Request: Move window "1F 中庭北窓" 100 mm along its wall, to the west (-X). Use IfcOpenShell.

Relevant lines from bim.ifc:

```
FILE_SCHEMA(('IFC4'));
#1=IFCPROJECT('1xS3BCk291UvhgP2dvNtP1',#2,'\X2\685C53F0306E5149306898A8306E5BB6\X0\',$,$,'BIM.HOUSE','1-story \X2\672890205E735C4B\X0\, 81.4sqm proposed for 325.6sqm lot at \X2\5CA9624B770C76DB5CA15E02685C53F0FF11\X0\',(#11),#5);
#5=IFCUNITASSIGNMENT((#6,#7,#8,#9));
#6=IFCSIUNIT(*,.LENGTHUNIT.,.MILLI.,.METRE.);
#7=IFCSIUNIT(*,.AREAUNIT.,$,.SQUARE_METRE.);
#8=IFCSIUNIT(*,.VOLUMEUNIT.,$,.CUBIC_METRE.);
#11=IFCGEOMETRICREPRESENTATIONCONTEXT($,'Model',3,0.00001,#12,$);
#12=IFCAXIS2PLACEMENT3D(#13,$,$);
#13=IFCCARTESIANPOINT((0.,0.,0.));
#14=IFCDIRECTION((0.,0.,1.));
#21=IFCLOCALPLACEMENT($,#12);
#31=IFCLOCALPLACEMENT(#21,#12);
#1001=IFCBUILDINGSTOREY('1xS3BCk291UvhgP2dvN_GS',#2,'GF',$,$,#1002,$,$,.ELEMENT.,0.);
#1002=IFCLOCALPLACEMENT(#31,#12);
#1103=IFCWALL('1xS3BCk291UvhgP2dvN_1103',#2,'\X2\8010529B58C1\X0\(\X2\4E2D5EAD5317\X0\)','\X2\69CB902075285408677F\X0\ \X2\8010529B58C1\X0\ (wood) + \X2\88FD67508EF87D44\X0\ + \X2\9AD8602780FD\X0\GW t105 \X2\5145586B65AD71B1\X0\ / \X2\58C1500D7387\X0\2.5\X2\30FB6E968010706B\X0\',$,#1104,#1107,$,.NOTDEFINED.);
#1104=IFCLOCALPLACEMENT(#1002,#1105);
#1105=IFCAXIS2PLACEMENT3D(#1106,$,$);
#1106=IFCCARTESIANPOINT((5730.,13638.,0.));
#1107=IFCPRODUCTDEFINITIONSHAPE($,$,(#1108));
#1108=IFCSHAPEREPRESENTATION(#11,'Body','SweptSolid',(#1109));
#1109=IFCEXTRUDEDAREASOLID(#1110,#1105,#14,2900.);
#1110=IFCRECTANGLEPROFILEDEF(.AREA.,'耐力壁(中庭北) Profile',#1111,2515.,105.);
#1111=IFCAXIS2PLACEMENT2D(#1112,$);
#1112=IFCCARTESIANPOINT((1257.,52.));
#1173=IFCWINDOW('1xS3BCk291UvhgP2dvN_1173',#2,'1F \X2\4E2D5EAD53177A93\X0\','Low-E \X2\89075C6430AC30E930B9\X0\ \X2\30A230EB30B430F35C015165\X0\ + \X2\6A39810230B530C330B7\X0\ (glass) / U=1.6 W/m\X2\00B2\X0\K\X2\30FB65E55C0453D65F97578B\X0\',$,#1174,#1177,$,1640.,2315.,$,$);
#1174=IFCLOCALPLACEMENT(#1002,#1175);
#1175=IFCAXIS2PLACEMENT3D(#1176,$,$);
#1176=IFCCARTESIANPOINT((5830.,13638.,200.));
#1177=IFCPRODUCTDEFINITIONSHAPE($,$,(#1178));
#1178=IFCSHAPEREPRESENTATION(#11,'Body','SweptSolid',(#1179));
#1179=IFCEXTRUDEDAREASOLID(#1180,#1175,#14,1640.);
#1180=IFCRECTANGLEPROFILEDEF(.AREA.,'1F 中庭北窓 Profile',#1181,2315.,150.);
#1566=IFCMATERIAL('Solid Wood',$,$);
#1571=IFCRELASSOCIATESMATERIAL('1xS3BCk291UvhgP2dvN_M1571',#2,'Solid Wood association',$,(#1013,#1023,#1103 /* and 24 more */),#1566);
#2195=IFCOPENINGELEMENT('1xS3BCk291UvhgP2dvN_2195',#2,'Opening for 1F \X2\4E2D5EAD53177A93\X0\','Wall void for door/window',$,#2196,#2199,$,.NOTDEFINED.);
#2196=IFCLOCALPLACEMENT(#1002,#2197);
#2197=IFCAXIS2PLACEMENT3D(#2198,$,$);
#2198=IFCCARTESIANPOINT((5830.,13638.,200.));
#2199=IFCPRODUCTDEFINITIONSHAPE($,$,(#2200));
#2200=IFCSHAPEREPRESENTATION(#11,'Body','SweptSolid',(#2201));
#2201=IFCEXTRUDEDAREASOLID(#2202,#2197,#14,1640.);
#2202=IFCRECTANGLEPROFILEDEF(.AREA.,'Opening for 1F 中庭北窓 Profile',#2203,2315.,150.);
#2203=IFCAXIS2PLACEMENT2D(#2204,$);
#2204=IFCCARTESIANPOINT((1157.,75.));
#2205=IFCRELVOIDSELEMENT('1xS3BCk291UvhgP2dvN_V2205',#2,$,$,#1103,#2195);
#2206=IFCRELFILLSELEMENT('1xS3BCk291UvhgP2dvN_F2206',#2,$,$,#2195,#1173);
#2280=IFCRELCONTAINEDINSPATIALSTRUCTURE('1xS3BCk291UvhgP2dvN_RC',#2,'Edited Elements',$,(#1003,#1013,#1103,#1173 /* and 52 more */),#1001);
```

```python
import ifcopenshell
import ifcopenshell.api.geometry
import ifcopenshell.util.placement

model = ifcopenshell.open("bim.ifc")

window = model.by_id(1173)
opening = window.FillsVoids[0].RelatingOpeningElement
wall = opening.VoidsElements[0].RelatingBuildingElement

wall_matrix = ifcopenshell.util.placement.get_local_placement(wall.ObjectPlacement)
shift = wall_matrix[:3, 0] * -100.0
before = ifcopenshell.util.placement.get_local_placement(window.ObjectPlacement)[:3, 3].copy()

# The window is not placed relative to its opening, so move both.
for product in (opening, window):
    matrix = ifcopenshell.util.placement.get_local_placement(product.ObjectPlacement)
    matrix[:3, 3] += shift
    ifcopenshell.api.geometry.edit_object_placement(model, product=product, matrix=matrix, is_si=False)

after = ifcopenshell.util.placement.get_local_placement(window.ObjectPlacement)[:3, 3]
print("window moved by", (after - before).round(3) + 0.0)

model.write("bim_edited.ifc")
```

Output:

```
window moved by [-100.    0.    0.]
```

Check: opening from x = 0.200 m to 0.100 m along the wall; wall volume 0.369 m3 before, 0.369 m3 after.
